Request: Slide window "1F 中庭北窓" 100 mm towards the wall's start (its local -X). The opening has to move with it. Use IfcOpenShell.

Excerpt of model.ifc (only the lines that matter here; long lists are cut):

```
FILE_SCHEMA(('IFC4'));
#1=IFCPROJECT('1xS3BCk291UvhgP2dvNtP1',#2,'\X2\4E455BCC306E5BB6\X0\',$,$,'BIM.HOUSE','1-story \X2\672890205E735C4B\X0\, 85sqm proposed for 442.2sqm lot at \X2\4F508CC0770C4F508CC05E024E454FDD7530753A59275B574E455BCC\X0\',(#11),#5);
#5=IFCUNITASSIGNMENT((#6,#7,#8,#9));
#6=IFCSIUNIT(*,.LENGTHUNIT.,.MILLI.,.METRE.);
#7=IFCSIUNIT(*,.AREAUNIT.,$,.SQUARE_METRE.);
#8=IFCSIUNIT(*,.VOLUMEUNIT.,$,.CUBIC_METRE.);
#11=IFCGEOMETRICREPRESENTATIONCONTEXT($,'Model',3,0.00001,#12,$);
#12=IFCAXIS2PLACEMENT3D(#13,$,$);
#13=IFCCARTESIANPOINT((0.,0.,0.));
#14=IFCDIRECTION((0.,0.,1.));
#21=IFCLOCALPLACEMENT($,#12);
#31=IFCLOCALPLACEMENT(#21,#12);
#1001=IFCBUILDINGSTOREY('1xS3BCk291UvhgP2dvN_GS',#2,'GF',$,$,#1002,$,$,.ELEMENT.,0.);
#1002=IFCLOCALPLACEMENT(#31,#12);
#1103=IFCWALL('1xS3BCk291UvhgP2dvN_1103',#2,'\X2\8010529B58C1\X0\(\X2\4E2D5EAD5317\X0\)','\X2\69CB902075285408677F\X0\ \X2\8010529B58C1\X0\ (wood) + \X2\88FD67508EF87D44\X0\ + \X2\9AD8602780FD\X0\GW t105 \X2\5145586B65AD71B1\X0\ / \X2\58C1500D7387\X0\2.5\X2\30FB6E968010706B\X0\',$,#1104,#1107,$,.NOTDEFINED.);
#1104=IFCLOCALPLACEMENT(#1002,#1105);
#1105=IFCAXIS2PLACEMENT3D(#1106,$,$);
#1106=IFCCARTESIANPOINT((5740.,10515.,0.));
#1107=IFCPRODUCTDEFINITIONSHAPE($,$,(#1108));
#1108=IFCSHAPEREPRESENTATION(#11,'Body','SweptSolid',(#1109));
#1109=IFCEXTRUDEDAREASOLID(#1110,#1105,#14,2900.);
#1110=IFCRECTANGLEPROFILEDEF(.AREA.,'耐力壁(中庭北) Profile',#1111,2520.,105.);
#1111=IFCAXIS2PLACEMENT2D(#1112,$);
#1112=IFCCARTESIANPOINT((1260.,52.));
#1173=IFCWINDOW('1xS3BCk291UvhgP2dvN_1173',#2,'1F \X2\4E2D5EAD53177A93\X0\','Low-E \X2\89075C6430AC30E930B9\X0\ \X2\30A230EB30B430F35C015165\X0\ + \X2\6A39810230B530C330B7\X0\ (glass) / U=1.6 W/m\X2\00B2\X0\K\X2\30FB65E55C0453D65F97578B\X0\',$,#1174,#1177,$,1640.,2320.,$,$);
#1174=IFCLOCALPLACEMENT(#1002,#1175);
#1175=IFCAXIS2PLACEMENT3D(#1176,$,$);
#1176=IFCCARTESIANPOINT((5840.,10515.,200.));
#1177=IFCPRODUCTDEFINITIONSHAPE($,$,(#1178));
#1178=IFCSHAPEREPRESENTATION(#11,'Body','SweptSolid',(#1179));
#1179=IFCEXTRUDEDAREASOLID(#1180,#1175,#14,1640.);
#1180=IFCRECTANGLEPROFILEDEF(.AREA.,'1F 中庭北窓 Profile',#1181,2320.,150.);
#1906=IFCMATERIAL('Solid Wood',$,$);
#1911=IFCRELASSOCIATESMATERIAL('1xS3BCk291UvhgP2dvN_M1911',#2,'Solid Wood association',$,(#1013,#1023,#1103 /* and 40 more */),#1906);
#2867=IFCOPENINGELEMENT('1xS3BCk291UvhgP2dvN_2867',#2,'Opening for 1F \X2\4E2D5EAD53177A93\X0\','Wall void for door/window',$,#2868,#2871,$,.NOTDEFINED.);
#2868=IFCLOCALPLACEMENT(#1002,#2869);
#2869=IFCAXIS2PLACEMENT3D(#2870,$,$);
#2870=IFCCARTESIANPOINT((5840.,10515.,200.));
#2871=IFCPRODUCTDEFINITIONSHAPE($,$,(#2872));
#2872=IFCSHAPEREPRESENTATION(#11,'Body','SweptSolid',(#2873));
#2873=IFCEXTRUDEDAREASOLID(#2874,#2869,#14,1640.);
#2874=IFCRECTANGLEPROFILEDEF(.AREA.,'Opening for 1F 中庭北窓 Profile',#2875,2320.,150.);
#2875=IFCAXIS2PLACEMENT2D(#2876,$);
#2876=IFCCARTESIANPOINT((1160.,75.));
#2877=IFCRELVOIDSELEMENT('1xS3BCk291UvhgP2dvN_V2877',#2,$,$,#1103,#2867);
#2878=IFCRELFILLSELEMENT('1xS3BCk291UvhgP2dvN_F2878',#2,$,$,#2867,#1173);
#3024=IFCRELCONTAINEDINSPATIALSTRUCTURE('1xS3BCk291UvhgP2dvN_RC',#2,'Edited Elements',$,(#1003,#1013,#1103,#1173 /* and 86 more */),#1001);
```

```python
import ifcopenshell
import ifcopenshell.api.geometry
import ifcopenshell.util.placement
import ifcopenshell.util.unit

model = ifcopenshell.open("model.ifc")
unit_scale = ifcopenshell.util.unit.calculate_unit_scale(model)

window = model.by_guid("1xS3BCk291UvhgP2dvN_1173")
opening = window.FillsVoids[0].RelatingOpeningElement
wall = opening.VoidsElements[0].RelatingBuildingElement

wall_matrix = ifcopenshell.util.placement.get_local_placement(wall.ObjectPlacement)
shift = wall_matrix[:3, 0] * -0.1 / unit_scale
before = ifcopenshell.util.placement.get_local_placement(window.ObjectPlacement)[:3, 3].copy()

# The window is not placed relative to its opening, so move both.
for product in (opening, window):
    matrix = ifcopenshell.util.placement.get_local_placement(product.ObjectPlacement)
    matrix[:3, 3] += shift
    ifcopenshell.api.geometry.edit_object_placement(model, product=product, matrix=matrix, is_si=False)

after = ifcopenshell.util.placement.get_local_placement(window.ObjectPlacement)[:3, 3]
print("window moved by", (after - before).round(3) + 0.0)

model.write("model_rev.ifc")
```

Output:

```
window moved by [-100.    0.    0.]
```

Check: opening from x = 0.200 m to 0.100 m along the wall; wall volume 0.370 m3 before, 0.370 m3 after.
